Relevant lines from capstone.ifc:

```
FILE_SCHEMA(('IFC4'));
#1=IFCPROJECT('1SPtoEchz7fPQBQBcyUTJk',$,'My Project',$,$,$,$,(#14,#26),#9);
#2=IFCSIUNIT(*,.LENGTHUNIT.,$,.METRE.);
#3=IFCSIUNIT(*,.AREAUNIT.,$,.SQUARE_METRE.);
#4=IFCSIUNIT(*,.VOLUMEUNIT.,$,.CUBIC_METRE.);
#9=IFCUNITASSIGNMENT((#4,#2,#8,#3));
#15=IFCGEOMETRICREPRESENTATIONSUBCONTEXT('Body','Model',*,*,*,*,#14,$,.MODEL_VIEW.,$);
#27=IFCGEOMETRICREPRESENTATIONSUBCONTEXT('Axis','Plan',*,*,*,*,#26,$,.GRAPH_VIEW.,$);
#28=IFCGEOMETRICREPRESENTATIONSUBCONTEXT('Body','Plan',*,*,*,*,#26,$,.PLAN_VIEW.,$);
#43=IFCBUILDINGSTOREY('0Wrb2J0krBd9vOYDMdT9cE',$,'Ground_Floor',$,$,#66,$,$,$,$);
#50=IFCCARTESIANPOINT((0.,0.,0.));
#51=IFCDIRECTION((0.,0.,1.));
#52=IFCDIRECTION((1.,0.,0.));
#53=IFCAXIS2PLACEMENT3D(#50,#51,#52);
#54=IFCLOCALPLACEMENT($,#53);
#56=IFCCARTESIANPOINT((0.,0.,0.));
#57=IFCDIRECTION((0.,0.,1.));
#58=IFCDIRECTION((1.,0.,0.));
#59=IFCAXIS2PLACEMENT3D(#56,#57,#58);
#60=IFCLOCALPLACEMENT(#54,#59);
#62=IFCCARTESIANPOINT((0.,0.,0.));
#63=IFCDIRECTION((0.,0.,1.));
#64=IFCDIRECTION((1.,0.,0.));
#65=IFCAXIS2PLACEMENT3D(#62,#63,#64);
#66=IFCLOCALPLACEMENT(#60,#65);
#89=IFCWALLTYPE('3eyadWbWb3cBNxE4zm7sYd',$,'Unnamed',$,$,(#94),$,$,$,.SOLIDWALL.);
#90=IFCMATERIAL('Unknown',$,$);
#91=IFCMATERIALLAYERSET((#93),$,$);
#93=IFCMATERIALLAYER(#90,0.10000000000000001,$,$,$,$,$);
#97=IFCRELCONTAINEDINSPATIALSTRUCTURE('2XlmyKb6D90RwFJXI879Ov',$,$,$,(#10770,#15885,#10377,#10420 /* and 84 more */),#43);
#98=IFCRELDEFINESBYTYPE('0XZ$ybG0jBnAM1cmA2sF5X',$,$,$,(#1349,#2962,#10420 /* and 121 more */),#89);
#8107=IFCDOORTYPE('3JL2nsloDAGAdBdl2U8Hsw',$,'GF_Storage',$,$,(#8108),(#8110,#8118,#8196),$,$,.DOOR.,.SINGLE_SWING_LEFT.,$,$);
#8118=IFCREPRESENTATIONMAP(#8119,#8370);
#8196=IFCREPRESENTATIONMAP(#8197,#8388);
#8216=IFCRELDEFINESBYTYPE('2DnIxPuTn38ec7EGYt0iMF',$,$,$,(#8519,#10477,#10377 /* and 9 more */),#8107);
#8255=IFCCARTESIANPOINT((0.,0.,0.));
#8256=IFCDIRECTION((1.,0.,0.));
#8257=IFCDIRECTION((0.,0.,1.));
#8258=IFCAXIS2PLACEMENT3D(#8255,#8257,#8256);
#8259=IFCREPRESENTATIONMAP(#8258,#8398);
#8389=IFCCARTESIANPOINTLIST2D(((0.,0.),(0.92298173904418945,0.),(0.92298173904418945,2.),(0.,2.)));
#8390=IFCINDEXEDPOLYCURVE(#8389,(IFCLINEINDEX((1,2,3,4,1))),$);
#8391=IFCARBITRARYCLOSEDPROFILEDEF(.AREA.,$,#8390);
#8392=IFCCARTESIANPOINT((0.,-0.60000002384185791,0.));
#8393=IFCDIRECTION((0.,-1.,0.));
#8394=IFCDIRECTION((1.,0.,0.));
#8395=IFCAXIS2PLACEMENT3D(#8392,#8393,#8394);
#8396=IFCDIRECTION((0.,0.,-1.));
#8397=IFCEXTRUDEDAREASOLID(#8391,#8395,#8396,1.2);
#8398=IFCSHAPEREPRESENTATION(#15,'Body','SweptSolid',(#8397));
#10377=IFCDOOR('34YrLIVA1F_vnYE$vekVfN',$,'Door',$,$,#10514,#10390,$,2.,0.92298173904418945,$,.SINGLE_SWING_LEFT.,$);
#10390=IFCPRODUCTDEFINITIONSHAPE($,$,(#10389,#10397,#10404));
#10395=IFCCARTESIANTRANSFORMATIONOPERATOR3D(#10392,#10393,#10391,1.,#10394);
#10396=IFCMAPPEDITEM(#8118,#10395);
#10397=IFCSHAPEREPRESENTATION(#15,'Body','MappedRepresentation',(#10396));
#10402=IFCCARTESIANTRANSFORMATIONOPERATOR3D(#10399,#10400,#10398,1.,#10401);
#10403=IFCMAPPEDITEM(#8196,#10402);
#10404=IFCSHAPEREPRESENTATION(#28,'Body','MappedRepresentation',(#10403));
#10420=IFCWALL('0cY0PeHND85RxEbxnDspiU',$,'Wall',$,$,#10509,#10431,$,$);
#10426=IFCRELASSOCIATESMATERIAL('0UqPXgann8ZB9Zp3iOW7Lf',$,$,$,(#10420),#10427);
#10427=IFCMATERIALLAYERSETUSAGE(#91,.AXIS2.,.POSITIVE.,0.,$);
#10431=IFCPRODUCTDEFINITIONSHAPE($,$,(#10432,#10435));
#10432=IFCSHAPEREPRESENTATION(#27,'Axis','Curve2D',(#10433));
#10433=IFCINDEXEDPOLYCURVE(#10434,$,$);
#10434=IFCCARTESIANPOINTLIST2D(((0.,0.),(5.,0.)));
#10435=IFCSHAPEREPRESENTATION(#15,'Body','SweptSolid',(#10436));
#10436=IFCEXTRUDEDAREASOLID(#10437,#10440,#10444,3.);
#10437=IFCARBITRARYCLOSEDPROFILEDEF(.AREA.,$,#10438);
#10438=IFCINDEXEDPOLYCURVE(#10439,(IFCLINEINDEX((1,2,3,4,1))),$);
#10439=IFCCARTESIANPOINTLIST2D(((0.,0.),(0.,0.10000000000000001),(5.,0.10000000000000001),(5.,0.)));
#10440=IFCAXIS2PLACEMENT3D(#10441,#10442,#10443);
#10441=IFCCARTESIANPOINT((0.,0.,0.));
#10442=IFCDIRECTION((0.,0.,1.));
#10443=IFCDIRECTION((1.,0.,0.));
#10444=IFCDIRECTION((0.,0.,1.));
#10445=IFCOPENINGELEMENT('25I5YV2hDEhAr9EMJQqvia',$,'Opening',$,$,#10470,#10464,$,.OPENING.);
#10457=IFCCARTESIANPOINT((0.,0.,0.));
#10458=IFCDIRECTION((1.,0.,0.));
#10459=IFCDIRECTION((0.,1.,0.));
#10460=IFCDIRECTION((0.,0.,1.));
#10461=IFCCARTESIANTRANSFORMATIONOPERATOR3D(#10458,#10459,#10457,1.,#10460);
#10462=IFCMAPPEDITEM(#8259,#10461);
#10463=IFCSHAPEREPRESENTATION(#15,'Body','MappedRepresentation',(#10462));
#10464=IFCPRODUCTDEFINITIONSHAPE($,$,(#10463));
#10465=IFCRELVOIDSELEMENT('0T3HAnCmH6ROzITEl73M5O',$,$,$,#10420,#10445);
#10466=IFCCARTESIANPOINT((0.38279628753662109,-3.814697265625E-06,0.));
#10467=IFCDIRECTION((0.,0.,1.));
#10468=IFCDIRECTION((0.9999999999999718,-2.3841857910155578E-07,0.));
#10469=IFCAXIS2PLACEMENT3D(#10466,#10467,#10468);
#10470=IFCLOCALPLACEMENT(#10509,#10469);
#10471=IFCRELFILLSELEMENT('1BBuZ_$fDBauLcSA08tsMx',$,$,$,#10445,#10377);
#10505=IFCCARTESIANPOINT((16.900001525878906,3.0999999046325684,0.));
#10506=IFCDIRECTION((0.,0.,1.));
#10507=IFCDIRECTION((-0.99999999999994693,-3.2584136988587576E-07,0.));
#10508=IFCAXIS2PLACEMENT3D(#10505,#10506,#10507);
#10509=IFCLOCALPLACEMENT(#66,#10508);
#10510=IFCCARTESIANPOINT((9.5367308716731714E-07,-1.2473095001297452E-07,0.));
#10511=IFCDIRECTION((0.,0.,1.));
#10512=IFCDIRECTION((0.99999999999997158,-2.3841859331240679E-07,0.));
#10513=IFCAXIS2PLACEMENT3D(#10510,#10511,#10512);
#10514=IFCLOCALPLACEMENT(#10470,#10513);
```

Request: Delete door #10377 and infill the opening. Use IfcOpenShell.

```python
import ifcopenshell
import ifcopenshell.api.feature
import ifcopenshell.api.root
import ifcopenshell.geom
import ifcopenshell.util.shape

model = ifcopenshell.open("capstone.ifc")
settings = ifcopenshell.geom.settings()


def volume(element):
    """Net volume in cubic metres, openings subtracted."""
    shape = ifcopenshell.geom.create_shape(settings, element)
    return ifcopenshell.util.shape.get_volume(shape.geometry)


door = model.by_guid("34YrLIVA1F_vnYE$vekVfN")
opening = door.FillsVoids[0].RelatingOpeningElement
wall = opening.VoidsElements[0].RelatingBuildingElement
before = volume(wall)

ifcopenshell.api.root.remove_product(model, product=door)
ifcopenshell.api.feature.remove_feature(model, feature=opening)

after = volume(wall)

print(f"wall volume {before:.3f} -> {after:.3f} m3")

model.write("capstone_updated.ifc")
```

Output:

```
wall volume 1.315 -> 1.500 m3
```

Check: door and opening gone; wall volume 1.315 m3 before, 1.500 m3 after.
